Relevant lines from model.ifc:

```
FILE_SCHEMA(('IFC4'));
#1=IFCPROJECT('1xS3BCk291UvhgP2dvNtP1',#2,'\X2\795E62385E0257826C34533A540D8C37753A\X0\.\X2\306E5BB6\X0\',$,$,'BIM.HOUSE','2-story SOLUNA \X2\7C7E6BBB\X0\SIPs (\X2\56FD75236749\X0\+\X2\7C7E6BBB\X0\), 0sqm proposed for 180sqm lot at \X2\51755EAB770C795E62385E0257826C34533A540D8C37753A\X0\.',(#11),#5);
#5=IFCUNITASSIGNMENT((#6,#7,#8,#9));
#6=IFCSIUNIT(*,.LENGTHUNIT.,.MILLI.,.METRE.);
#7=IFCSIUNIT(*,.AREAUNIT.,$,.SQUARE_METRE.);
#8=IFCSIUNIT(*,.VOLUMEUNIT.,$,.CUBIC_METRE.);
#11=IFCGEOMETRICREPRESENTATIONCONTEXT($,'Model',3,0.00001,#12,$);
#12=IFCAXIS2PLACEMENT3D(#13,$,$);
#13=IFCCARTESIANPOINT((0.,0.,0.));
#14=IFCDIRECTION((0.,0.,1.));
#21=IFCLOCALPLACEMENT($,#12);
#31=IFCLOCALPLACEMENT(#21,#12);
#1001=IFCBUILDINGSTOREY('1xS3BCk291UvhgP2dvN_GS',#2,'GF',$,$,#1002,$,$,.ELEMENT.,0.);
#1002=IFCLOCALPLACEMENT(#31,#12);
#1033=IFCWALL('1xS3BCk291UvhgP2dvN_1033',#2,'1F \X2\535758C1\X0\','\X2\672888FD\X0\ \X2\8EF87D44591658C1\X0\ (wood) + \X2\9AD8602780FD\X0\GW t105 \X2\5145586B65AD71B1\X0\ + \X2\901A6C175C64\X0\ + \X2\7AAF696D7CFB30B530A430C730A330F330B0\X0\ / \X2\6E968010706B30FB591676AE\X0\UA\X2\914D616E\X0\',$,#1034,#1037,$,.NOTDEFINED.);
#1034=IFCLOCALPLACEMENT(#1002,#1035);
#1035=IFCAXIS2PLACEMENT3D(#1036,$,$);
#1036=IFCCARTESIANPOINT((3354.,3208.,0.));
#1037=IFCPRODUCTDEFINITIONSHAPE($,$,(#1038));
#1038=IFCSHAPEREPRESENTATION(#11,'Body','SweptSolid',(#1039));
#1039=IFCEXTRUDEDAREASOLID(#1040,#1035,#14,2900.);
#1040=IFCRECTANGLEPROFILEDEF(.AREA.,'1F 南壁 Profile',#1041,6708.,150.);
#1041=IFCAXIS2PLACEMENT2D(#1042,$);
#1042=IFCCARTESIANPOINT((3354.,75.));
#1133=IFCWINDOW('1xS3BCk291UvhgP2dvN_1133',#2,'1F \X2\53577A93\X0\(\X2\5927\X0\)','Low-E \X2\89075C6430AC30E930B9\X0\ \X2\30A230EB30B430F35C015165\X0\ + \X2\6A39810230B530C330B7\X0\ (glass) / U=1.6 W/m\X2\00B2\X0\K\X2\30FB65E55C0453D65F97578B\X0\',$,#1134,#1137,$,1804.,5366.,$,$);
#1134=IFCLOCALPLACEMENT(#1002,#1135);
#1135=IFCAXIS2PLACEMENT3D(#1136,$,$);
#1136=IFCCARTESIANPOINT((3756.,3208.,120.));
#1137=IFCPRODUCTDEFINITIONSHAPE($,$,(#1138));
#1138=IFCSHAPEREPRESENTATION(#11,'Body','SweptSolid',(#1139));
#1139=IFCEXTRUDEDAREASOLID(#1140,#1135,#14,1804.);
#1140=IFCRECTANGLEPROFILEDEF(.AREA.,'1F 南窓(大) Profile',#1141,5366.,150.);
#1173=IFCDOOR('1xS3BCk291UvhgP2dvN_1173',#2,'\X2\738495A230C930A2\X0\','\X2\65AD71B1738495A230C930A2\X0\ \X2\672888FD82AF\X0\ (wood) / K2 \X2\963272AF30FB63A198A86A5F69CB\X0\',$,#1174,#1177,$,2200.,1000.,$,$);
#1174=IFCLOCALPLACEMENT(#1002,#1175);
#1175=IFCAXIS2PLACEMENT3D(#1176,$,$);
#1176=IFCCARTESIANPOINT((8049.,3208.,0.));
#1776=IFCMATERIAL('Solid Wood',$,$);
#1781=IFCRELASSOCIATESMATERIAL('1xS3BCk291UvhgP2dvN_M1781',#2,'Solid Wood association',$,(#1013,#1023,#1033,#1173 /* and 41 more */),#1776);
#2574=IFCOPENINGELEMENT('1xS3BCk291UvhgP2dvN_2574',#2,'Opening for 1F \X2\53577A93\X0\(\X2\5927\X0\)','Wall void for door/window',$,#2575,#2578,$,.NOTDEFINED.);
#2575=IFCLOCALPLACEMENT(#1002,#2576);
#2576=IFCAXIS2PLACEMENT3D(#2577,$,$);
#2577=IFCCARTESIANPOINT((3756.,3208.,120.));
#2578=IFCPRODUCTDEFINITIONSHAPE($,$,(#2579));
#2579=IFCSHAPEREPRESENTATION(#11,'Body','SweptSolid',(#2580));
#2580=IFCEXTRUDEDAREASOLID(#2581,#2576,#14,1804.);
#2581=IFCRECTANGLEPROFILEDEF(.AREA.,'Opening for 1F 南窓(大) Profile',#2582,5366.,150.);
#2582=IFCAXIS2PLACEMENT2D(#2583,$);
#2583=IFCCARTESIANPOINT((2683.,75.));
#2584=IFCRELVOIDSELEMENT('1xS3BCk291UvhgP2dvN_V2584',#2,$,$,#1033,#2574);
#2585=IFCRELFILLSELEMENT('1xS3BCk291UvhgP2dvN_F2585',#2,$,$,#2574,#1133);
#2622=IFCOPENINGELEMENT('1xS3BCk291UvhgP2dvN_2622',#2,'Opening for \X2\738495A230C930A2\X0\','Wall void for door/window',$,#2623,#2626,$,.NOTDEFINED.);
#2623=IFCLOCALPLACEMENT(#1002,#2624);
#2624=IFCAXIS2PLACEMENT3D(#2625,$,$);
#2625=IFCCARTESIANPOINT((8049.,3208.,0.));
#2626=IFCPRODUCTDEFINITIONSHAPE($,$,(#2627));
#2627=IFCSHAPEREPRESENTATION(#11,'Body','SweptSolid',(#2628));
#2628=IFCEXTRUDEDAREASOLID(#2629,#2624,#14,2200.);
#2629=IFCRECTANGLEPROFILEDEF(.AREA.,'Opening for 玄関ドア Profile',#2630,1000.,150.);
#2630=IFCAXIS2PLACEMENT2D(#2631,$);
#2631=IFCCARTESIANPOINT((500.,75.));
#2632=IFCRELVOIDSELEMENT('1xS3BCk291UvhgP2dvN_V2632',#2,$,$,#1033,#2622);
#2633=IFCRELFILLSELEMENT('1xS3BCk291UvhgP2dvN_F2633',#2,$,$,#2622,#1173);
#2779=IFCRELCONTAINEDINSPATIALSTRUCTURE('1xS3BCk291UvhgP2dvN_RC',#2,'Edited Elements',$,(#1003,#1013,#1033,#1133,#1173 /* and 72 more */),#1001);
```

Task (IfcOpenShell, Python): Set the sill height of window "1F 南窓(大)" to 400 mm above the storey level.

```python
import numpy as np
import ifcopenshell
import ifcopenshell.api.geometry
import ifcopenshell.geom
import ifcopenshell.util.element
import ifcopenshell.util.placement
import ifcopenshell.util.shape
import ifcopenshell.util.unit

model = ifcopenshell.open("model.ifc")
unit_scale = ifcopenshell.util.unit.calculate_unit_scale(model)

window = model.by_guid("1xS3BCk291UvhgP2dvN_1133")
opening = window.FillsVoids[0].RelatingOpeningElement
storey = ifcopenshell.util.element.get_container(window, ifc_class="IfcBuildingStorey")
level = ifcopenshell.util.placement.get_local_placement(storey.ObjectPlacement)[2, 3]

# The opening's origin need not be at the sill, so measure its lowest point.
shape = ifcopenshell.geom.create_shape(ifcopenshell.geom.settings(), opening)
bottom = ifcopenshell.util.shape.get_shape_bottom_elevation(shape, shape.geometry) / unit_scale
dz = level + 0.4 / unit_scale - bottom

shift = np.array([0.0, 0.0, dz])
# The window is not placed relative to its opening, so move both.
for product in (opening, window):
    matrix = ifcopenshell.util.placement.get_local_placement(product.ObjectPlacement)
    matrix[:3, 3] += shift
    ifcopenshell.api.geometry.edit_object_placement(model, product=product, matrix=matrix, is_si=False)

print(f"moved by {dz * unit_scale:+.3f} m")

model.write("model_rev.ifc")
```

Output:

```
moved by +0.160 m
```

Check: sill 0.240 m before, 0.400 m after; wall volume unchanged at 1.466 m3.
